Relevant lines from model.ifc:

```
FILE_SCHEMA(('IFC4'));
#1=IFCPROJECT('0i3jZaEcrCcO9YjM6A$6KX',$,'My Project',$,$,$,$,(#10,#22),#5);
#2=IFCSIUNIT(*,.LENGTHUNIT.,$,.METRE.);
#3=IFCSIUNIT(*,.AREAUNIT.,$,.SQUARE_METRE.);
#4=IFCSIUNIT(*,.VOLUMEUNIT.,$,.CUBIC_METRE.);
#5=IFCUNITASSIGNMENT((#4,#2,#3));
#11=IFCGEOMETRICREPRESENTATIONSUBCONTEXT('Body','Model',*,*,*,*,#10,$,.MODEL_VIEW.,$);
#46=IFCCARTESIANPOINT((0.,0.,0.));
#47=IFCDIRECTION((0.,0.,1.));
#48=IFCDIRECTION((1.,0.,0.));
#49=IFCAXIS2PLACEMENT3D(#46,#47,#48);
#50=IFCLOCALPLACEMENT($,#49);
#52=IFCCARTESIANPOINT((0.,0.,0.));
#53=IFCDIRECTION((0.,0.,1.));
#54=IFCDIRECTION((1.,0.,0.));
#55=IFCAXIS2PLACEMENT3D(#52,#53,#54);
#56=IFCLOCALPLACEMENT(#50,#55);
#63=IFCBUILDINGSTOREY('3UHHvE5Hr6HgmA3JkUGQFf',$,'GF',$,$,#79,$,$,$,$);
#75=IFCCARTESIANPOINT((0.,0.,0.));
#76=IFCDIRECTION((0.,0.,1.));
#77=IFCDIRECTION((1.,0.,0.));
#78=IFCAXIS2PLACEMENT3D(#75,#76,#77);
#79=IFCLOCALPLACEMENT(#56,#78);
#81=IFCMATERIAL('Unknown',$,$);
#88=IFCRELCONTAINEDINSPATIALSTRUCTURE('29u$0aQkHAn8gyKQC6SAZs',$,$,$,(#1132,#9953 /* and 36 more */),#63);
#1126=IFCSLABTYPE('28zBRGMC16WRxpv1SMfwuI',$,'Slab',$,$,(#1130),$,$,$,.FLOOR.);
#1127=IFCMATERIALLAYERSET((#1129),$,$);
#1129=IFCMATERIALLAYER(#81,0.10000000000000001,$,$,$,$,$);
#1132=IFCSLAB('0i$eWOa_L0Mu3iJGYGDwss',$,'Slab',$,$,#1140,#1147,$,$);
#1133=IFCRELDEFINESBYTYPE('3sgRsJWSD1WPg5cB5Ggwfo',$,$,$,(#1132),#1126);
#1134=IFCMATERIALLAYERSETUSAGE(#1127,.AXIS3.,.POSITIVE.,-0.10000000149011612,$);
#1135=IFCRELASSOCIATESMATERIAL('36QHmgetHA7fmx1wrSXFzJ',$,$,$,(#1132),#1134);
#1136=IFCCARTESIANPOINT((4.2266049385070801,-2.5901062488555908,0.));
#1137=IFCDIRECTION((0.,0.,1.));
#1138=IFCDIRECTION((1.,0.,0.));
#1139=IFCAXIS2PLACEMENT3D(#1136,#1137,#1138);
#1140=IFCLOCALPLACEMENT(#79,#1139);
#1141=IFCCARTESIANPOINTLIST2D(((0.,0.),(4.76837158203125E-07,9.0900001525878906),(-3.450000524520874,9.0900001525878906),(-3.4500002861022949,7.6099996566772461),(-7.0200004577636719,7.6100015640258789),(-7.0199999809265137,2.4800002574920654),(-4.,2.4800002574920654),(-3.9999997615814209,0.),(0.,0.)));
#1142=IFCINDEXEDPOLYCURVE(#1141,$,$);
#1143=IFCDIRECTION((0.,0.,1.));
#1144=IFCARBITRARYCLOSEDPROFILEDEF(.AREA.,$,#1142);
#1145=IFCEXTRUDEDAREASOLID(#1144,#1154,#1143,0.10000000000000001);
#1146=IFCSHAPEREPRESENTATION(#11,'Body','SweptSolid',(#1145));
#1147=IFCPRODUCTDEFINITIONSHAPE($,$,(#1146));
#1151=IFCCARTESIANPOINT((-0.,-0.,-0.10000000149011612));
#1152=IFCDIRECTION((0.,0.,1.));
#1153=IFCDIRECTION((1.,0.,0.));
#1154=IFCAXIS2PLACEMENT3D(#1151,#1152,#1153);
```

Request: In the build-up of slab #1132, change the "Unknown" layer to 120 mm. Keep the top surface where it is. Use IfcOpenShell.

```python
import ifcopenshell
import ifcopenshell.util.element
import ifcopenshell.util.representation
import ifcopenshell.util.unit

model = ifcopenshell.open("model.ifc")
unit_scale = ifcopenshell.util.unit.calculate_unit_scale(model)

layer_set = model.by_id(1127)
layer = next(l for l in layer_set.MaterialLayers if l.Material and l.Material.Name == "Unknown")
change = 0.12 / unit_scale - layer.LayerThickness
layer.LayerThickness += change

# Geometry does not follow the layer set by itself.
slabs = [e for e in ifcopenshell.util.element.get_elements_by_material(model, layer_set) if e.is_a("IfcSlab")]
for slab in sorted(slabs, key=lambda e: e.id()):
    body = ifcopenshell.util.representation.get_representation(slab, "Model", "Body")
    solid = body.Items[0]
    old_depth = solid.Depth
    solid.Depth += change
    # Extruded upwards: lower the start of the extrusion so the top stays.
    x, y, z = solid.Position.Location.Coordinates
    solid.Position.Location = model.createIfcCartesianPoint((x, y, z - change))
    print(slab.id(), f"{old_depth:g} -> {solid.Depth:g}")

# The layers are counted up from the underside, which has moved.
for usage in {ifcopenshell.util.element.get_material(slab) for slab in slabs}:
    usage.OffsetFromReferenceLine -= change

model.write("model_edited.ifc")
```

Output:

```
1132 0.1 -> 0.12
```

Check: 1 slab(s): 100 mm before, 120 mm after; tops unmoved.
